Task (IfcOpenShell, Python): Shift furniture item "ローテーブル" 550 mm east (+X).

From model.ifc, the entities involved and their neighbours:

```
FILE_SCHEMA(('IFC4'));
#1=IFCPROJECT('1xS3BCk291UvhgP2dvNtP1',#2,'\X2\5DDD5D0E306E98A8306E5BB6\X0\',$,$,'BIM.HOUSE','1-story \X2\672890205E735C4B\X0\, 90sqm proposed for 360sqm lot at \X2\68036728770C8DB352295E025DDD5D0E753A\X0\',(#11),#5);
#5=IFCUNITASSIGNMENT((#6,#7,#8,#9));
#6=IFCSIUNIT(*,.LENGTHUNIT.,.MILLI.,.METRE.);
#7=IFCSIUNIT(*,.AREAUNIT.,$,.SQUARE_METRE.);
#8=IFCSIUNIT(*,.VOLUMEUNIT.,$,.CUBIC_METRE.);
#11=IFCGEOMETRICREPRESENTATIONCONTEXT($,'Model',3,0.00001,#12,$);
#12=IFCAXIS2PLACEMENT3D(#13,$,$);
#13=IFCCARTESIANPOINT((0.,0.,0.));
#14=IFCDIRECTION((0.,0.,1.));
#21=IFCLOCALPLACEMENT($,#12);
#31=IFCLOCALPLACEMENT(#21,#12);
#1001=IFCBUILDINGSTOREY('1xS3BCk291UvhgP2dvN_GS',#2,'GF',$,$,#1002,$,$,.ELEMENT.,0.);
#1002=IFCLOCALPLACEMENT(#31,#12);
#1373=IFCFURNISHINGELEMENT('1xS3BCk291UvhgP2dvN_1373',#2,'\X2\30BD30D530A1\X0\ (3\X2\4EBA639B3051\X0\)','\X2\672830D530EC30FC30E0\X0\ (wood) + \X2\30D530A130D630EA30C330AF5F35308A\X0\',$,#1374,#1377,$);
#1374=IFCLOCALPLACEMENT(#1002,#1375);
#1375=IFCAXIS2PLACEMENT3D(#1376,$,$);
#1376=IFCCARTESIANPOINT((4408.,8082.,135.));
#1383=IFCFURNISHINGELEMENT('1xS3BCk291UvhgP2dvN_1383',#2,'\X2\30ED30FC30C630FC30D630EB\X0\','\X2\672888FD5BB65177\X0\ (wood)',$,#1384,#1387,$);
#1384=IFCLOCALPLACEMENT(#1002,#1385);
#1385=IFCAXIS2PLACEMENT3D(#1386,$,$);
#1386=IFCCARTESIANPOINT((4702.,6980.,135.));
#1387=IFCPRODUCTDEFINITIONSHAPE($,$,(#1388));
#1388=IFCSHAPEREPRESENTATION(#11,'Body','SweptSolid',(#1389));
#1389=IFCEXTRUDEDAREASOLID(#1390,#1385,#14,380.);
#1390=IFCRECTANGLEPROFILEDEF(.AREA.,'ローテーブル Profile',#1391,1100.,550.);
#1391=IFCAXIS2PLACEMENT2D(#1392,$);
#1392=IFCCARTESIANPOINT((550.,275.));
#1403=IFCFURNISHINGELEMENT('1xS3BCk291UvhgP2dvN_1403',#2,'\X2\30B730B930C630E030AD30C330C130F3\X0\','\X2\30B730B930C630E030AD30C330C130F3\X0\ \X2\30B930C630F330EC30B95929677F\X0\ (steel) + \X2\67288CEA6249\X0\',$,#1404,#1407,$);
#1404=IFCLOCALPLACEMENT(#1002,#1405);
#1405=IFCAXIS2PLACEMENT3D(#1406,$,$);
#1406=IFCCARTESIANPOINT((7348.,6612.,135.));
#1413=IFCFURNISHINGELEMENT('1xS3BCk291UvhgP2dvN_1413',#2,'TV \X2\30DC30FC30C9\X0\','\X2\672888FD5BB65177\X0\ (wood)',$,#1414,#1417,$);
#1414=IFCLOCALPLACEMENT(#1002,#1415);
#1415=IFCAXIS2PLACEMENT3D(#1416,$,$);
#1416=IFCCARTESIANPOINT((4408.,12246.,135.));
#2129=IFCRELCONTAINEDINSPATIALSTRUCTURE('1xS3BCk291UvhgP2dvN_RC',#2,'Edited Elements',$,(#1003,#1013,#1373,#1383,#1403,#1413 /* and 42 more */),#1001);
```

```python
import ifcopenshell
import ifcopenshell.api.geometry
import ifcopenshell.util.placement
import ifcopenshell.util.unit

model = ifcopenshell.open("model.ifc")
unit_scale = ifcopenshell.util.unit.calculate_unit_scale(model)

item = model.by_id(1383)
matrix = ifcopenshell.util.placement.get_local_placement(item.ObjectPlacement)
matrix[0, 3] += 0.55 / unit_scale
ifcopenshell.api.geometry.edit_object_placement(model, product=item, matrix=matrix, is_si=False)

print(ifcopenshell.util.placement.get_local_placement(item.ObjectPlacement).round(3) + 0.0)

model.write("model_edited.ifc")
```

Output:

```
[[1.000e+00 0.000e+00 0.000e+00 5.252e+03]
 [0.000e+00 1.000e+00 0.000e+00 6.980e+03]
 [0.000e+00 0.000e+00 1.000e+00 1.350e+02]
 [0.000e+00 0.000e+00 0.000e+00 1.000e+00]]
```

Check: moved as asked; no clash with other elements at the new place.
